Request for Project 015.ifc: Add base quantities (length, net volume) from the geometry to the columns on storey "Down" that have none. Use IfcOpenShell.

First a look at what the model holds.

```python
import ifcopenshell
import ifcopenshell.util.element
import ifcopenshell.util.unit

model = ifcopenshell.open("Project 015.ifc")
print(model.schema)
for unit_type in ("LENGTHUNIT", "AREAUNIT", "VOLUMEUNIT"):
    print(unit_type, ifcopenshell.util.unit.calculate_unit_scale(model, unit_type))
storey = next(s for s in model.by_type("IfcBuildingStorey") if s.Name == "Down")
columns = [e for e in ifcopenshell.util.element.get_decomposition(storey) if e.is_a("IfcColumn")]
for e in sorted(columns, key=lambda e: e.id()):
    print(e.id(), e.is_a(), e.Name, list(ifcopenshell.util.element.get_psets(e, qtos_only=True)), sep=" | ")
```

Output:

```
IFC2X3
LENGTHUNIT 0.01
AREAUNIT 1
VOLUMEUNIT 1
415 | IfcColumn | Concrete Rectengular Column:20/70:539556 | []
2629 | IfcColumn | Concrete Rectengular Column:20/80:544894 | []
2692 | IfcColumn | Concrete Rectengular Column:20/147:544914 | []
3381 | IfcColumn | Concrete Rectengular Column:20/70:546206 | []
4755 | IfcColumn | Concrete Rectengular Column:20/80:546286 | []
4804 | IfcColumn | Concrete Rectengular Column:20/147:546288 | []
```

```python
import ifcopenshell
import ifcopenshell.api.pset
import ifcopenshell.geom
import ifcopenshell.util.element
import ifcopenshell.util.shape
import ifcopenshell.util.unit

model = ifcopenshell.open("Project 015.ifc")
unit_scale = ifcopenshell.util.unit.calculate_unit_scale(model)
volume_scale = ifcopenshell.util.unit.calculate_unit_scale(model, "VOLUMEUNIT")
settings = ifcopenshell.geom.settings()

storey = next(s for s in model.by_type("IfcBuildingStorey") if s.Name == "Down")
columns = [e for e in ifcopenshell.util.element.get_decomposition(storey) if e.is_a("IfcColumn")]

for e in sorted(columns, key=lambda e: e.id()):
    if ifcopenshell.util.element.get_psets(e, qtos_only=True, should_inherit=False):
        continue
    # Geometry comes back in metres, in the element's own axes.
    shape = ifcopenshell.geom.create_shape(settings, e)
    values = {
        "Length": ifcopenshell.util.shape.get_z(shape.geometry) / unit_scale,
        "NetVolume": ifcopenshell.util.shape.get_volume(shape.geometry) / volume_scale,
    }
    qto = ifcopenshell.api.pset.add_qto(model, product=e, name="BaseQuantities")
    ifcopenshell.api.pset.edit_qto(model, qto=qto, properties=values)
    print(e.id(), {k: round(v, 3) for k, v in values.items()})

model.write("Project 015_edited.ifc")
```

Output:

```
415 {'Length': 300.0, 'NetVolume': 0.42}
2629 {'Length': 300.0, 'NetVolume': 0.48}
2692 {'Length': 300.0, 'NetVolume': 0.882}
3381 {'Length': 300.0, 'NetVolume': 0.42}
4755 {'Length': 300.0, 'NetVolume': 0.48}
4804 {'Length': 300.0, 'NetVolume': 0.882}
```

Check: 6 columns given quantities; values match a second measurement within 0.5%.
